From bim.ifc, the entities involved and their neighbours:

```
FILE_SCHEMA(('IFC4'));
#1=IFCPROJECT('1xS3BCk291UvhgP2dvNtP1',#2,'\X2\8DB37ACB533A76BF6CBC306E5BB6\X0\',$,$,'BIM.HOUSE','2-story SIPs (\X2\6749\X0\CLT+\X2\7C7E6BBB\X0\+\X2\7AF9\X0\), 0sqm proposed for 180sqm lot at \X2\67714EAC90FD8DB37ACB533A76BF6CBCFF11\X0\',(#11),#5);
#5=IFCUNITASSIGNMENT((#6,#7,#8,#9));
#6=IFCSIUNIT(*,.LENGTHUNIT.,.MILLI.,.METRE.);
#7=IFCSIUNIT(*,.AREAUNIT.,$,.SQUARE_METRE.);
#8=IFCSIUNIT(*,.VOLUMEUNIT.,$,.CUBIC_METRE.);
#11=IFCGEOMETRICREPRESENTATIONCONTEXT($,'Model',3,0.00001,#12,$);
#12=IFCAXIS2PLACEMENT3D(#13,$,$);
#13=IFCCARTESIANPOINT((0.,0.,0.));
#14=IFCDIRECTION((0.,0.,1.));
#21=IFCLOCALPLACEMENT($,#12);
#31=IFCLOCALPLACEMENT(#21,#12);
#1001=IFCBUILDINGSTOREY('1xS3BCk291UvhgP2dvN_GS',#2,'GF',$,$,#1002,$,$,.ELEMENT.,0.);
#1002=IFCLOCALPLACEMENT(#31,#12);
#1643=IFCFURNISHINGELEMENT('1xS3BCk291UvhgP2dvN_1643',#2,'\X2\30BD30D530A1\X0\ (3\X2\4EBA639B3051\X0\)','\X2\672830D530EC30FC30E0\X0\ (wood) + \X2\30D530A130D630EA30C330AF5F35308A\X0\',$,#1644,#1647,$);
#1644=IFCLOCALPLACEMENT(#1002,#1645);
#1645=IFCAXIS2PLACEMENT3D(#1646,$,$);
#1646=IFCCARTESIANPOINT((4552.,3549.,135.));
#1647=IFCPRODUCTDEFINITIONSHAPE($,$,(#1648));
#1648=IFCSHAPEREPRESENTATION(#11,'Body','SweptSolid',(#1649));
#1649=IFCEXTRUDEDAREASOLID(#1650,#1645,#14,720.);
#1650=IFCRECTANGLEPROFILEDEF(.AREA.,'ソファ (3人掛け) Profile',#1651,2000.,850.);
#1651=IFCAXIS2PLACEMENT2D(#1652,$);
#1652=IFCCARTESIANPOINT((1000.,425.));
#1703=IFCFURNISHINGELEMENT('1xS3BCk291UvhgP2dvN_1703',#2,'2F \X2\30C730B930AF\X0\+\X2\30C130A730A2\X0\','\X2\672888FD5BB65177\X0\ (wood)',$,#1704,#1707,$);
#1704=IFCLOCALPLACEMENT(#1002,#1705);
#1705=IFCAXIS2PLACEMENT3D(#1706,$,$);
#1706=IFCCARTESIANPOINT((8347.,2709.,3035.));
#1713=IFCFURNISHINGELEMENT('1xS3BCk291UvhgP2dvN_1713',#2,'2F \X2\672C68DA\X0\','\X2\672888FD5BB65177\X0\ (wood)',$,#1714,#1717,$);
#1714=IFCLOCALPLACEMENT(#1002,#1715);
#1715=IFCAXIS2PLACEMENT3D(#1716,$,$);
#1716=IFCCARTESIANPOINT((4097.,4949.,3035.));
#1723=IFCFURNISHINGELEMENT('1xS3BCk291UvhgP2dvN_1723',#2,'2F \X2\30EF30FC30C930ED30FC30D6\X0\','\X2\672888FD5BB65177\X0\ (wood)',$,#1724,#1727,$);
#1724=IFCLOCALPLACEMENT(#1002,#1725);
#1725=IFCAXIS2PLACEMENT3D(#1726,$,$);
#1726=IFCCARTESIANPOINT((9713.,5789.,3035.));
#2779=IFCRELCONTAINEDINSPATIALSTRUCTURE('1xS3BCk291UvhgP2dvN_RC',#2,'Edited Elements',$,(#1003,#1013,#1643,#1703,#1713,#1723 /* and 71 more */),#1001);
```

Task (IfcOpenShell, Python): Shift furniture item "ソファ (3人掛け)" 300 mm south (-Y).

```python
import ifcopenshell
import ifcopenshell.api.geometry
import ifcopenshell.util.placement

model = ifcopenshell.open("bim.ifc")

item = model.by_guid("1xS3BCk291UvhgP2dvN_1643")
matrix = ifcopenshell.util.placement.get_local_placement(item.ObjectPlacement)
matrix[1, 3] -= 300.0
ifcopenshell.api.geometry.edit_object_placement(model, product=item, matrix=matrix, is_si=False)

print(ifcopenshell.util.placement.get_local_placement(item.ObjectPlacement).round(3) + 0.0)

model.write("bim_updated.ifc")
```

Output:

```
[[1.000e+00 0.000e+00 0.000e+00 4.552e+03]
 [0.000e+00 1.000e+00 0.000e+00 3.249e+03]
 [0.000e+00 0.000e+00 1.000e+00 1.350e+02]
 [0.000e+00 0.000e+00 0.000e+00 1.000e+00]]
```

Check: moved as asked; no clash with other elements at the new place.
